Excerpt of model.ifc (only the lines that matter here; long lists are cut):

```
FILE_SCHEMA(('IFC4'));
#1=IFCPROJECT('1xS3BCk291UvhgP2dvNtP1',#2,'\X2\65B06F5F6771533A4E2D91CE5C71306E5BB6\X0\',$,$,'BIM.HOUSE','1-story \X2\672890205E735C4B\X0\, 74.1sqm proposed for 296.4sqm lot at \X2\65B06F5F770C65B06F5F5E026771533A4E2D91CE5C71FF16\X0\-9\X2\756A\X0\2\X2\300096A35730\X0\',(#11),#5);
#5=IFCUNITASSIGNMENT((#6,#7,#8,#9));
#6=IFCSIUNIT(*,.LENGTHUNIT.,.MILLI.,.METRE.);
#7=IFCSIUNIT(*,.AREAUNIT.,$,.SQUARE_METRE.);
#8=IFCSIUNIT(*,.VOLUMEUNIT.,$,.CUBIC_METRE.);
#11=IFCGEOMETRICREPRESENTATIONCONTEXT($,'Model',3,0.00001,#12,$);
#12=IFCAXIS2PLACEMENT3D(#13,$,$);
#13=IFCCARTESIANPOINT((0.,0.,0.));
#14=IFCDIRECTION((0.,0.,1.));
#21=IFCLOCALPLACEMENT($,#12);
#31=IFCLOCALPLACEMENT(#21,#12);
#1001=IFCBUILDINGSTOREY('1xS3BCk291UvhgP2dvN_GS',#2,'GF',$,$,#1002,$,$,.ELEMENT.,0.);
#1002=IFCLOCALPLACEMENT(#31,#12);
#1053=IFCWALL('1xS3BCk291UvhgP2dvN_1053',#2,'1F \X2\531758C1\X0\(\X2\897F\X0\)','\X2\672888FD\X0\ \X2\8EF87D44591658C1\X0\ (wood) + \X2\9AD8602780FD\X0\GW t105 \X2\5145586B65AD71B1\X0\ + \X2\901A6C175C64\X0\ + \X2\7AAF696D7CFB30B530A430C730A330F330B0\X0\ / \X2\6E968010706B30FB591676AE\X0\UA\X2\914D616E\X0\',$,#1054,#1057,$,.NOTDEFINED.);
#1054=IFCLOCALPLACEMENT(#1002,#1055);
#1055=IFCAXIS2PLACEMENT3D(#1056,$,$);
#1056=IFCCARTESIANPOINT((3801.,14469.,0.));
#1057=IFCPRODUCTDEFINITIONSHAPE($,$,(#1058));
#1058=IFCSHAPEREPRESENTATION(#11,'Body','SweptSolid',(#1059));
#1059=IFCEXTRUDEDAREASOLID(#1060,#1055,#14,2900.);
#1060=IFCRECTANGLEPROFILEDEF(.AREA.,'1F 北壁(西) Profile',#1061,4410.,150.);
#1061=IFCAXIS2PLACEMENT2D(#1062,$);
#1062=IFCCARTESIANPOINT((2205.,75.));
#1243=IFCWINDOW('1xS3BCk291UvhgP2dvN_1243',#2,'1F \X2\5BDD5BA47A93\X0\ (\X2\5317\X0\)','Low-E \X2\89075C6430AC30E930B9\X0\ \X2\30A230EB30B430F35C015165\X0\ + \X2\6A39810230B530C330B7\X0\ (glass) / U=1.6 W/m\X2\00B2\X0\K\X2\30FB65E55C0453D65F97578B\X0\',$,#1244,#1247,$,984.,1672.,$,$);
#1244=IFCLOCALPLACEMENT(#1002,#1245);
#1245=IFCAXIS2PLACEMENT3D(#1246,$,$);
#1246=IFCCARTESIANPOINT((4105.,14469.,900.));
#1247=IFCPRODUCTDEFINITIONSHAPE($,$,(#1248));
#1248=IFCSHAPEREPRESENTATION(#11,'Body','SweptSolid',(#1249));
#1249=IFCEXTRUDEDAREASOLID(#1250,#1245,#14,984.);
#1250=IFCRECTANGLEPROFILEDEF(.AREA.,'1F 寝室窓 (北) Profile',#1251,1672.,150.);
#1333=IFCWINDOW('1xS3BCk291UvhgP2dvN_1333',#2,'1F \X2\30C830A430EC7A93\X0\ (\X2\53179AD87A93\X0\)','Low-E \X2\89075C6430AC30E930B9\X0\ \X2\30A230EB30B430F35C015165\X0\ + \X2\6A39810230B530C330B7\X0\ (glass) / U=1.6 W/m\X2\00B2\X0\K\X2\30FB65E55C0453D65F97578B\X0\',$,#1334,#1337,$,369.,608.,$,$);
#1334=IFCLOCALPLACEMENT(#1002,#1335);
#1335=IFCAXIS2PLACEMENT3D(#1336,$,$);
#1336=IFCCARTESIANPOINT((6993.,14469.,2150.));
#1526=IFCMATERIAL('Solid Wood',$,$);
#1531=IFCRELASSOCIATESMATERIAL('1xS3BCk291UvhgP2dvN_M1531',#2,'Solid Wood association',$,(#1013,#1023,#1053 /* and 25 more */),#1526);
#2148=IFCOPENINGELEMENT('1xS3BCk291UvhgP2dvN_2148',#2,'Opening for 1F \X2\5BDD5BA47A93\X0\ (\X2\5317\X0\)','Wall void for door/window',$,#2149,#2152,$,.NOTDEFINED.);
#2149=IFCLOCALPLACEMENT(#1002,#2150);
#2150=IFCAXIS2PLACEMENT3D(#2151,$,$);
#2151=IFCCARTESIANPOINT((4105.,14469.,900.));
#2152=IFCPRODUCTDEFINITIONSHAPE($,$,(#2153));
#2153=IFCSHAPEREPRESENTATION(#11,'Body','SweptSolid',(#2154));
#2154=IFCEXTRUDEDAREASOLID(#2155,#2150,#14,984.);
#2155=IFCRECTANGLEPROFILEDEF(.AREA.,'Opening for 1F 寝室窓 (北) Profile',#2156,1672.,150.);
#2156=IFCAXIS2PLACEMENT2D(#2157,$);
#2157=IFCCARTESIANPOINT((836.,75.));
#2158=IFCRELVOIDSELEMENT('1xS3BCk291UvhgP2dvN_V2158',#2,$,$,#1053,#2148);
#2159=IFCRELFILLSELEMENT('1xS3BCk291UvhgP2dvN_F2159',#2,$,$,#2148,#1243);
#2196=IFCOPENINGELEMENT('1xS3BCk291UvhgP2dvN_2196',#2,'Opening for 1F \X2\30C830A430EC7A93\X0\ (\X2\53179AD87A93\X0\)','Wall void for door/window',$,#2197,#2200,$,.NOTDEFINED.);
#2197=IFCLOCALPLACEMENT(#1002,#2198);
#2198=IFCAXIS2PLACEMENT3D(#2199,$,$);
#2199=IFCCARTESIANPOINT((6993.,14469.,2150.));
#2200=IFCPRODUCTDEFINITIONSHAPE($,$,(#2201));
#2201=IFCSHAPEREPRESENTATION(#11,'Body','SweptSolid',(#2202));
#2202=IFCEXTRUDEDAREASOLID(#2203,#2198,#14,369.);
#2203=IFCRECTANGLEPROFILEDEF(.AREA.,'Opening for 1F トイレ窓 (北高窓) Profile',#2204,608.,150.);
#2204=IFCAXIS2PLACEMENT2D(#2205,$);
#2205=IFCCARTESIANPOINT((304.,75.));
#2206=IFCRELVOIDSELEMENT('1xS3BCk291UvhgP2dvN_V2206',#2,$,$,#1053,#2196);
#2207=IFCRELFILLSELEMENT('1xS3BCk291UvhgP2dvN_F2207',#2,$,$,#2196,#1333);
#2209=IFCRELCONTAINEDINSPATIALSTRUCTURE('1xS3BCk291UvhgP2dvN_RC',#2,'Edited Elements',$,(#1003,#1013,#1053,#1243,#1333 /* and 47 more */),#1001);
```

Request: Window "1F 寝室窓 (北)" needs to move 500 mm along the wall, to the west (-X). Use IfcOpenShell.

```python
import ifcopenshell
import ifcopenshell.api.geometry
import ifcopenshell.util.placement

model = ifcopenshell.open("model.ifc")

window = model.by_guid("1xS3BCk291UvhgP2dvN_1243")
opening = window.FillsVoids[0].RelatingOpeningElement
wall = opening.VoidsElements[0].RelatingBuildingElement

wall_matrix = ifcopenshell.util.placement.get_local_placement(wall.ObjectPlacement)
shift = wall_matrix[:3, 0] * -500.0
before = ifcopenshell.util.placement.get_local_placement(window.ObjectPlacement)[:3, 3].copy()

# The window is not placed relative to its opening, so move both.
for product in (opening, window):
    matrix = ifcopenshell.util.placement.get_local_placement(product.ObjectPlacement)
    matrix[:3, 3] += shift
    ifcopenshell.api.geometry.edit_object_placement(model, product=product, matrix=matrix, is_si=False)

after = ifcopenshell.util.placement.get_local_placement(window.ObjectPlacement)[:3, 3]
print("window moved by", (after - before).round(3) + 0.0)

model.write("model_rev.ifc")
```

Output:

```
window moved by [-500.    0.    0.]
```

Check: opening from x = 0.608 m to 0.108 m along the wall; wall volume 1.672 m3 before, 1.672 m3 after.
